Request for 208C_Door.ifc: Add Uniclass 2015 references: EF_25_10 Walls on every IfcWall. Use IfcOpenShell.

First a look at what the model holds.

```python
import ifcopenshell

model = ifcopenshell.open("208C_Door.ifc")
print(model.schema)
print("classifications:", [c.Name for c in model.by_type("IfcClassification")])
for ifc_class in ("IfcDoor", "IfcRoof", "IfcStair", "IfcWall", "IfcWindow"):
    print(ifc_class, len(model.by_type(ifc_class)))
```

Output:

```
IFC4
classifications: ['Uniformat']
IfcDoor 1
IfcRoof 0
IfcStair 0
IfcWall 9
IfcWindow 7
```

```python
import ifcopenshell
import ifcopenshell.api.classification

model = ifcopenshell.open("208C_Door.ifc")

system = ifcopenshell.api.classification.add_classification(model, classification="Uniclass 2015")

codes = {
    "IfcWall": ("EF_25_10", "Walls"),
}
for ifc_class, (code, name) in codes.items():
    products = model.by_type(ifc_class)
    ifcopenshell.api.classification.add_reference(
        model, products=products, classification=system, identification=code, name=name
    )
    print(code, len(products))

model.write("208C_Door_edited.ifc")
```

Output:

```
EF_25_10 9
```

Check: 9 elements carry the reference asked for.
